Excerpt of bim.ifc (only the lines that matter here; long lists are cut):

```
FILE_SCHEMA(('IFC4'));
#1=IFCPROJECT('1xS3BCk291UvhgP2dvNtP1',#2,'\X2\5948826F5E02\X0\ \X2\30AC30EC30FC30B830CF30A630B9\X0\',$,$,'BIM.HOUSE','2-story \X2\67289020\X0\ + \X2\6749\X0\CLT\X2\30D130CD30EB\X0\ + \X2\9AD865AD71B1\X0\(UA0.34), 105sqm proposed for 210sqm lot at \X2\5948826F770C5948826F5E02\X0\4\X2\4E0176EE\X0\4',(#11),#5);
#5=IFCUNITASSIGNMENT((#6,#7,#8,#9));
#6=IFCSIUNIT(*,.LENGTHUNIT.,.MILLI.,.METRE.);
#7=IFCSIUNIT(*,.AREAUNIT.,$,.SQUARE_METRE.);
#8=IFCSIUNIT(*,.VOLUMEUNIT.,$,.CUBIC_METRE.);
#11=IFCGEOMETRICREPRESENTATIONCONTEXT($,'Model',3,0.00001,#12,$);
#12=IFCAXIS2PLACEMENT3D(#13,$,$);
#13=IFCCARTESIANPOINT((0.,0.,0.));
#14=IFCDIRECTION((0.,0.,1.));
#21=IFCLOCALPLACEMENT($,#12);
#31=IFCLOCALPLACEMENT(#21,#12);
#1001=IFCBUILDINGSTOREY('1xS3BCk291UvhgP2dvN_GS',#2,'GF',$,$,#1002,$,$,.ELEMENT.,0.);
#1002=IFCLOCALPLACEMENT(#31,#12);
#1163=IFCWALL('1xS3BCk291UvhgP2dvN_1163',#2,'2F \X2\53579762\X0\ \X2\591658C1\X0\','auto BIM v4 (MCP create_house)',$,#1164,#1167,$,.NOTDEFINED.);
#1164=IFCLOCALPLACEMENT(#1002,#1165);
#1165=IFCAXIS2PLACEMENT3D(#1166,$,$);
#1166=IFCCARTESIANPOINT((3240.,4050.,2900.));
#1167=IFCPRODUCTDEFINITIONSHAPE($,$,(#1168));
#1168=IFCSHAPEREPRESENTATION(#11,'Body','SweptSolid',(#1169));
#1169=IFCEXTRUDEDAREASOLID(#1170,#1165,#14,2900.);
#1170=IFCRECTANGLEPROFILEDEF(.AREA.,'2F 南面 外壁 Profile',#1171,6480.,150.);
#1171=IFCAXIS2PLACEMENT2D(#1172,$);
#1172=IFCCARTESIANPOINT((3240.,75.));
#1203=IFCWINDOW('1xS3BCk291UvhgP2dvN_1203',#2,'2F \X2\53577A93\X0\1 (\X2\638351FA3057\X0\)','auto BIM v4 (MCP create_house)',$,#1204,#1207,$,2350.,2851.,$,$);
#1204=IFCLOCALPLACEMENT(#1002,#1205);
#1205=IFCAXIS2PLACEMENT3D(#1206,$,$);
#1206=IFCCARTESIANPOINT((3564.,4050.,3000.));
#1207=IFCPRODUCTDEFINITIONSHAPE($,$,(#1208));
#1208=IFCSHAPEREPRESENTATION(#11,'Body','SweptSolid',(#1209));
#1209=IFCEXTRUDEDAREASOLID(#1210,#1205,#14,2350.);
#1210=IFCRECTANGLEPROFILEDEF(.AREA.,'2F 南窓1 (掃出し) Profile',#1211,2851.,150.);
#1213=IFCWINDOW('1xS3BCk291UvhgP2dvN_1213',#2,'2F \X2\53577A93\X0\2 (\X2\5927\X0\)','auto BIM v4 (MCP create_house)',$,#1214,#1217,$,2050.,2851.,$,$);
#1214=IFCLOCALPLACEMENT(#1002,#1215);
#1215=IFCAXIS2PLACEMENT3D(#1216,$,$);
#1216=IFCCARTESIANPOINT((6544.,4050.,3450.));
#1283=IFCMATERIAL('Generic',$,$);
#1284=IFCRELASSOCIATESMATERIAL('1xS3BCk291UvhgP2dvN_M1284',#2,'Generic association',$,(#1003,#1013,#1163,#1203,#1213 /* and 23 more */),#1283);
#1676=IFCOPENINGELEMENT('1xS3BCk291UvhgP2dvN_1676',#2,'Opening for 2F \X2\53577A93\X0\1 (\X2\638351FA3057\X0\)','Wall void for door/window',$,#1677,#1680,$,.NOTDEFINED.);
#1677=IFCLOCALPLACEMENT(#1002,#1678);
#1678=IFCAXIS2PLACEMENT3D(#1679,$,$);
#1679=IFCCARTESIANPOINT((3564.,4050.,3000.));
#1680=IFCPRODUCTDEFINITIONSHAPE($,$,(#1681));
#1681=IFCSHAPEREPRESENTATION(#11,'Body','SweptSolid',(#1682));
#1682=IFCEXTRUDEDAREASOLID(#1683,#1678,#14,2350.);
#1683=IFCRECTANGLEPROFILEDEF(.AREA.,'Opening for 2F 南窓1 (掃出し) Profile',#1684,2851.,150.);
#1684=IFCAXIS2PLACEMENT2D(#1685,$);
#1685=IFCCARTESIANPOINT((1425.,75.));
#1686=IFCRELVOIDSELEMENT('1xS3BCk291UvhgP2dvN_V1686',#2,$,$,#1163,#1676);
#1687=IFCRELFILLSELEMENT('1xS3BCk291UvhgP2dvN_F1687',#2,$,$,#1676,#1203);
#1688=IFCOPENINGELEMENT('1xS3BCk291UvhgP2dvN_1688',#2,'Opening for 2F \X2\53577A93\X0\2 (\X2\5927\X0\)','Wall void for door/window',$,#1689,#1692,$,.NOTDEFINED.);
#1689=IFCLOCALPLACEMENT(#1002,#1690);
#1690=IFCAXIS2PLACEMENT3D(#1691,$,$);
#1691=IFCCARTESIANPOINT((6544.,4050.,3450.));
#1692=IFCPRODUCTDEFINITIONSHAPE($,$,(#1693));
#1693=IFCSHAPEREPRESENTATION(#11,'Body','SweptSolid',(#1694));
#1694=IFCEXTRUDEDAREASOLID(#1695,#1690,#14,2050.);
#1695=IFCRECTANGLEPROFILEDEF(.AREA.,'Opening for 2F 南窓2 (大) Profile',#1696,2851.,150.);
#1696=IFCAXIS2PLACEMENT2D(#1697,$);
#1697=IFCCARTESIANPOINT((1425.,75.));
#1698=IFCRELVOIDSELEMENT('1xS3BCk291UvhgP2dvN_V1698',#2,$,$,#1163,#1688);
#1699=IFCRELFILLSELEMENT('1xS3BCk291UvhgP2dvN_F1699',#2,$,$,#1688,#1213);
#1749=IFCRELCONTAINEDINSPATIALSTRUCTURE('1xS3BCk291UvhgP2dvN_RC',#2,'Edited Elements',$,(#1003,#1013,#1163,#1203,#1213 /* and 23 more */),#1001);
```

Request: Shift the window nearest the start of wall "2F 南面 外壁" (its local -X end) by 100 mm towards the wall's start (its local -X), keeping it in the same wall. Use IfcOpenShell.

```python
import ifcopenshell
import ifcopenshell.api.geometry
import ifcopenshell.util.placement

model = ifcopenshell.open("bim.ifc")

window = model.by_id(1203)
opening = window.FillsVoids[0].RelatingOpeningElement
wall = opening.VoidsElements[0].RelatingBuildingElement

wall_matrix = ifcopenshell.util.placement.get_local_placement(wall.ObjectPlacement)
shift = wall_matrix[:3, 0] * -100.0
before = ifcopenshell.util.placement.get_local_placement(window.ObjectPlacement)[:3, 3].copy()

# The window is not placed relative to its opening, so move both.
for product in (opening, window):
    matrix = ifcopenshell.util.placement.get_local_placement(product.ObjectPlacement)
    matrix[:3, 3] += shift
    ifcopenshell.api.geometry.edit_object_placement(model, product=product, matrix=matrix, is_si=False)

after = ifcopenshell.util.placement.get_local_placement(window.ObjectPlacement)[:3, 3]
print("window moved by", (after - before).round(3) + 0.0)

model.write("bim_updated.ifc")
```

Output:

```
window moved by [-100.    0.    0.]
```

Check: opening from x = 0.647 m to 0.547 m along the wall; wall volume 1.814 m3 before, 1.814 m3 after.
